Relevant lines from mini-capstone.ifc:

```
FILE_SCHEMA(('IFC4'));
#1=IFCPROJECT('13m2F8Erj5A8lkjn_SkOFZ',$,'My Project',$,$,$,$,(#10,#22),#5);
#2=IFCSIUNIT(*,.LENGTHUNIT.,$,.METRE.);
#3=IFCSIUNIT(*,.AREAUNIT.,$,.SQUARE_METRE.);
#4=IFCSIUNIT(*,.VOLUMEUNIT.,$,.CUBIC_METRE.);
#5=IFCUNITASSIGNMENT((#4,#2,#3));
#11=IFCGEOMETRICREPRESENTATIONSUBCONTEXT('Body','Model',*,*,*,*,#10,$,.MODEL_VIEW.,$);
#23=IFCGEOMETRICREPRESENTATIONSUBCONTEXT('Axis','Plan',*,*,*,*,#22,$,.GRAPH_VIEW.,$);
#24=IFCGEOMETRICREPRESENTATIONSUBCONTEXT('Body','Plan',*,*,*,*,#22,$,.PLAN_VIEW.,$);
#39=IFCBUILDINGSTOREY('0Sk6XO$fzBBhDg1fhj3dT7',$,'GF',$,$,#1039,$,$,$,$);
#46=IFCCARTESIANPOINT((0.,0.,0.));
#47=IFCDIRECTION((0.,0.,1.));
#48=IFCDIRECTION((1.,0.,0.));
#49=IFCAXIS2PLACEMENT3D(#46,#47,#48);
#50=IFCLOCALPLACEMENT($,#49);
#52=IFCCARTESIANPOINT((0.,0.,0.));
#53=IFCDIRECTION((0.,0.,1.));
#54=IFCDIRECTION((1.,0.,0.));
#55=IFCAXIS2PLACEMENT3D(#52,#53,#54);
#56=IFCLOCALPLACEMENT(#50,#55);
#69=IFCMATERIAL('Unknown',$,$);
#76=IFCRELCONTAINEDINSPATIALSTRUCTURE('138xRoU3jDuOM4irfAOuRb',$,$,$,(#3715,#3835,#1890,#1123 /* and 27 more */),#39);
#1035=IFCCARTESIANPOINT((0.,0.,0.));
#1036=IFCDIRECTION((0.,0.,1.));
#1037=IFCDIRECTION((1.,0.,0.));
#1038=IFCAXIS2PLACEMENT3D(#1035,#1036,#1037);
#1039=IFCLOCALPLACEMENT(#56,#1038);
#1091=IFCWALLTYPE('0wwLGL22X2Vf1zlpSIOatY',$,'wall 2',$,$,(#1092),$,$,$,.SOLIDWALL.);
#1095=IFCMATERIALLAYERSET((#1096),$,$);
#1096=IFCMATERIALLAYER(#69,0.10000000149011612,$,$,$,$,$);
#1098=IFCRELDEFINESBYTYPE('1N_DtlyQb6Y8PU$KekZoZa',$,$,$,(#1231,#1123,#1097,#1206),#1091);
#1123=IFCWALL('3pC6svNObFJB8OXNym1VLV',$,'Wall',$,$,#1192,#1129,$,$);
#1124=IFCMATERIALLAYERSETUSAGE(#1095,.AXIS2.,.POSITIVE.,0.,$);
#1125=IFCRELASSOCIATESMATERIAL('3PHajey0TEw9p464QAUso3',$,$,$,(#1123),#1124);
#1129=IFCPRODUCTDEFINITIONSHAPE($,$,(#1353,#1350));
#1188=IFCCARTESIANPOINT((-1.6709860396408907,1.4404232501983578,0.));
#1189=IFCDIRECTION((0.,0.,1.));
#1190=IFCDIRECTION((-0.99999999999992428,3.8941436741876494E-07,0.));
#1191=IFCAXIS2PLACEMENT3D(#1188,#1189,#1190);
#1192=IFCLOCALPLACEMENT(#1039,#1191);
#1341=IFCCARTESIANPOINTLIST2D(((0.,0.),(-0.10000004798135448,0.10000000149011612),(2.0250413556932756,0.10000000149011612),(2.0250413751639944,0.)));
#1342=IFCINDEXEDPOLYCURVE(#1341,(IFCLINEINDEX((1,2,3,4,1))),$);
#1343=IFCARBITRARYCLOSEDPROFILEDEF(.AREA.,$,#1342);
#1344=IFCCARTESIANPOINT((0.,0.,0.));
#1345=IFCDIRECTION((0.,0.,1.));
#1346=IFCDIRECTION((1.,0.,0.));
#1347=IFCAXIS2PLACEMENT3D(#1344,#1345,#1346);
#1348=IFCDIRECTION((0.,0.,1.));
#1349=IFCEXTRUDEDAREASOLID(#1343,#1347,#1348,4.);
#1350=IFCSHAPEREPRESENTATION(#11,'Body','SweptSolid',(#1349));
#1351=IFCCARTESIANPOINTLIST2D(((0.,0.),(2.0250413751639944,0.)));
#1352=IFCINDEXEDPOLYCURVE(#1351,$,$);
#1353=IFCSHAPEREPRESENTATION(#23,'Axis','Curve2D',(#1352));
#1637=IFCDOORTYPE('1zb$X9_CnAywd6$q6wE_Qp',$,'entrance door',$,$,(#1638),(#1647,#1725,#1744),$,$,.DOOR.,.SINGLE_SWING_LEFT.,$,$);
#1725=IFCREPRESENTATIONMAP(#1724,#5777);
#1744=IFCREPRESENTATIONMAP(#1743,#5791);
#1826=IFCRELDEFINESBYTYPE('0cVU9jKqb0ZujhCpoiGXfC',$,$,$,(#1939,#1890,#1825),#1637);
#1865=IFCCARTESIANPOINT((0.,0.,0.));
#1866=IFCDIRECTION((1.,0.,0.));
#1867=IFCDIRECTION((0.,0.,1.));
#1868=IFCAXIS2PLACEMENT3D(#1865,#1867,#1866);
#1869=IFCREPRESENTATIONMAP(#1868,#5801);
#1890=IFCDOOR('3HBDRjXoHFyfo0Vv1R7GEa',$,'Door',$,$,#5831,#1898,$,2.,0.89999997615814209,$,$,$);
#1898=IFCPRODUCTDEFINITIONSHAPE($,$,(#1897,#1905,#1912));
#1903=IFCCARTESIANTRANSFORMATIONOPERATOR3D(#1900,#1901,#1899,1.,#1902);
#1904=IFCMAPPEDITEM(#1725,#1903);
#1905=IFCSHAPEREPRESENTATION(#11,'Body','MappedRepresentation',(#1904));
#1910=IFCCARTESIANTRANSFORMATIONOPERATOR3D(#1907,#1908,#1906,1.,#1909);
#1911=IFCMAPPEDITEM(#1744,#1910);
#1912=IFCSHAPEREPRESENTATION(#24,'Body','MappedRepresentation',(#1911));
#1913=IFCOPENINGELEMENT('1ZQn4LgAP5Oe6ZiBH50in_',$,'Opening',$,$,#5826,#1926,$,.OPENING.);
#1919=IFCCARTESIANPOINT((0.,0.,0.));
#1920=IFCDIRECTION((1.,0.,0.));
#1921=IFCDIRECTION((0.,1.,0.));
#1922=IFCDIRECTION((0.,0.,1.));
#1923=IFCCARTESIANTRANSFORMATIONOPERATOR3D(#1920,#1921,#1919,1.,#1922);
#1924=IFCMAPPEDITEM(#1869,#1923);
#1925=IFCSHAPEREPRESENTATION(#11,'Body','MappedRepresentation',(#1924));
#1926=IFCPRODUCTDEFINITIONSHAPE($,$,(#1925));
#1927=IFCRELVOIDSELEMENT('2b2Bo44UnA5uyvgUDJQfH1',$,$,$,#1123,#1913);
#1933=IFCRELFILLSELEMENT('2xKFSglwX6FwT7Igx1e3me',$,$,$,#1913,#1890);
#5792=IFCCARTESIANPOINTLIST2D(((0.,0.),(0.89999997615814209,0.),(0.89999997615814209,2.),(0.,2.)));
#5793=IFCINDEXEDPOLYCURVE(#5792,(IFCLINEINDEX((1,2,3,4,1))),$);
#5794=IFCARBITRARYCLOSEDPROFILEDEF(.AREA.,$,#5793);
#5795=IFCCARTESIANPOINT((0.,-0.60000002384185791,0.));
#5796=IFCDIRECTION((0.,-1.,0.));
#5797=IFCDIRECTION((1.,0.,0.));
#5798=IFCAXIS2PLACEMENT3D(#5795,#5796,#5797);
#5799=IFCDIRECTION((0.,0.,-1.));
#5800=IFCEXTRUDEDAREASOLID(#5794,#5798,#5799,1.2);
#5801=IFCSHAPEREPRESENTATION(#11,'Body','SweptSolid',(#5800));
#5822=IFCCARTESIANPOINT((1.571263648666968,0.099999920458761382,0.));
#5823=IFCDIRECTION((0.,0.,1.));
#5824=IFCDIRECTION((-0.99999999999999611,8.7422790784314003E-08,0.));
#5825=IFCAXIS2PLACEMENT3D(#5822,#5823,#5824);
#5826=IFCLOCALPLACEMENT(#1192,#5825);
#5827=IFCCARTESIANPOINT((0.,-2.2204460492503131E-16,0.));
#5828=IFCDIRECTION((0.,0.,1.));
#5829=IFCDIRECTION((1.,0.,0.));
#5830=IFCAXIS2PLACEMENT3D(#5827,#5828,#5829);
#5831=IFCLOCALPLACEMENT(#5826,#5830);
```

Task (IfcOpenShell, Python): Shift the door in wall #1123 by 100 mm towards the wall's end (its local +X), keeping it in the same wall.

```python
import ifcopenshell
import ifcopenshell.api.geometry
import ifcopenshell.util.placement

model = ifcopenshell.open("mini-capstone.ifc")

door = model.by_guid("3HBDRjXoHFyfo0Vv1R7GEa")
opening = door.FillsVoids[0].RelatingOpeningElement
wall = opening.VoidsElements[0].RelatingBuildingElement

wall_matrix = ifcopenshell.util.placement.get_local_placement(wall.ObjectPlacement)
shift = wall_matrix[:3, 0] * 0.1
before = ifcopenshell.util.placement.get_local_placement(door.ObjectPlacement)[:3, 3].copy()

# The door is placed relative to its opening, so it follows when the opening moves.
matrix = ifcopenshell.util.placement.get_local_placement(opening.ObjectPlacement)
matrix[:3, 3] += shift
ifcopenshell.api.geometry.edit_object_placement(
    model, product=opening, matrix=matrix, is_si=False, should_transform_children=True
)

after = ifcopenshell.util.placement.get_local_placement(door.ObjectPlacement)[:3, 3]
print("door moved by", (after - before).round(3) + 0.0)

model.write("mini-capstone_v2.ifc")
```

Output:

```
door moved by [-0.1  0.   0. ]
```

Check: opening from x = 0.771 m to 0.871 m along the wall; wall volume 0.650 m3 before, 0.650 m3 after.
